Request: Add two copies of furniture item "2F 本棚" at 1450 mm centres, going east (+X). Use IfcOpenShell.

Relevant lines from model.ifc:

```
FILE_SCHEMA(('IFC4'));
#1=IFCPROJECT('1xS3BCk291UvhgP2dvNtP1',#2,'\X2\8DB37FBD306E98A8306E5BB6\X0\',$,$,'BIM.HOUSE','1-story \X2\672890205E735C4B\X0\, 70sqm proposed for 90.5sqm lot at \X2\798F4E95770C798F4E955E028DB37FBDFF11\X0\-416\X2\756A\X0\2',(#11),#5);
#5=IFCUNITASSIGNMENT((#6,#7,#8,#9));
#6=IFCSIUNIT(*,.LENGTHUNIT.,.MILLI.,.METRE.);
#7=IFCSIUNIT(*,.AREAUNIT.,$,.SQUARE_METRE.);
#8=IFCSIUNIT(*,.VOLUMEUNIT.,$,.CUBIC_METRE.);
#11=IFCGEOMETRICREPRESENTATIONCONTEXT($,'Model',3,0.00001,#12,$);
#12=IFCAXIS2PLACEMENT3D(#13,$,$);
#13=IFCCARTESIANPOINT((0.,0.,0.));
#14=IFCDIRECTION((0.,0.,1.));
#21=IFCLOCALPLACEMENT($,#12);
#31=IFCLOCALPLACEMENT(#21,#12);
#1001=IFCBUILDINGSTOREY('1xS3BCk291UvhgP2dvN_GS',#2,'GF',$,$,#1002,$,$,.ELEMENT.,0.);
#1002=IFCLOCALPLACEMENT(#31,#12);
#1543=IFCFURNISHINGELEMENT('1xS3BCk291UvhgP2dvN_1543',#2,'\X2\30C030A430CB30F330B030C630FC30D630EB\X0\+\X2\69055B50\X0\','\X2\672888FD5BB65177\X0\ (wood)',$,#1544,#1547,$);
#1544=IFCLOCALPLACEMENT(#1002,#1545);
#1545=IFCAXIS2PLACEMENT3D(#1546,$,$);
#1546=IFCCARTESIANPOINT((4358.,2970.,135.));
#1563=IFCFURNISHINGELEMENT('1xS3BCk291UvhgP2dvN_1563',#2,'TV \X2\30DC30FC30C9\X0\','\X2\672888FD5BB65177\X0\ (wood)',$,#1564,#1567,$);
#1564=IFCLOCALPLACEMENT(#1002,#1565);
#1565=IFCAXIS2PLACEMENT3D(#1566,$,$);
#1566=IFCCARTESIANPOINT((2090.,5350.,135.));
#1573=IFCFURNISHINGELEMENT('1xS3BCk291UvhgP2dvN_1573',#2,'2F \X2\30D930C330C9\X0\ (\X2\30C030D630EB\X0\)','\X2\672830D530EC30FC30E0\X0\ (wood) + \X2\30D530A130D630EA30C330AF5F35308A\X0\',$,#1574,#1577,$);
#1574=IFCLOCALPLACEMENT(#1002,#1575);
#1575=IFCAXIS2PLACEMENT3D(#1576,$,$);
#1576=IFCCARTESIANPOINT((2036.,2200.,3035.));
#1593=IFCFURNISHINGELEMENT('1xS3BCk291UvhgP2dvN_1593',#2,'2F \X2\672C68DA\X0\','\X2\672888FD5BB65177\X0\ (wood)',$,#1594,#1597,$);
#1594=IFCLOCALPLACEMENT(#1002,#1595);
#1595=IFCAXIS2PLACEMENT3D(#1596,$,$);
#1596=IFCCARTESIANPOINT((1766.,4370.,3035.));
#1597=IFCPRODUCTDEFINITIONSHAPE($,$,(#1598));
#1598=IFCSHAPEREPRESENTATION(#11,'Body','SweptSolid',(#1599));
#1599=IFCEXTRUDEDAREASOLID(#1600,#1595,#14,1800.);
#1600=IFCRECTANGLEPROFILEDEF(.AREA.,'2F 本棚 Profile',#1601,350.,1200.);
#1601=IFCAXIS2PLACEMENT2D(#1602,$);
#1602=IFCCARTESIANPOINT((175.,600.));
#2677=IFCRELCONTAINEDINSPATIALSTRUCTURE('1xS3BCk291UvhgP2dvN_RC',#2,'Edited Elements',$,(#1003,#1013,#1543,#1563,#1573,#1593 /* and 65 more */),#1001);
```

```python
import numpy as np
import ifcopenshell
import ifcopenshell.api.geometry
import ifcopenshell.api.root
import ifcopenshell.util.element
import ifcopenshell.util.placement
import ifcopenshell.util.unit

model = ifcopenshell.open("model.ifc")
unit_scale = ifcopenshell.util.unit.calculate_unit_scale(model)


def reuse_history(source, copy):
    """copy_class also copies each property set's owner history, people and application; keep the originals."""
    for rel in copy.IsDefinedBy:
        if rel.is_a("IfcRelDefinesByProperties") and (history := rel.RelatingPropertyDefinition.OwnerHistory):
            rel.RelatingPropertyDefinition.OwnerHistory = source.OwnerHistory
            ifcopenshell.util.element.remove_deep2(model, history)


source = model.by_id(1593)
base = ifcopenshell.util.placement.get_local_placement(source.ObjectPlacement)
step = np.array([1.0, 0.0, 0.0]) * 1.45 / unit_scale

for i in range(1, 3):
    copy = ifcopenshell.api.root.copy_class(model, product=source)
    copy.Representation = ifcopenshell.util.element.copy_deep(
        model, source.Representation, exclude=["IfcGeometricRepresentationContext", "IfcRepresentationMap"]
    )
    reuse_history(source, copy)
    matrix = base.copy()
    matrix[:3, 3] += i * step
    print("added at", matrix[:3, 3].round(3) + 0.0)
    ifcopenshell.api.geometry.edit_object_placement(model, product=copy, matrix=matrix, is_si=False)

model.write("model_rev.ifc")
```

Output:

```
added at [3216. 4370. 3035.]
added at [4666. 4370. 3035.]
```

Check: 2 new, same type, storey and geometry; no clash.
